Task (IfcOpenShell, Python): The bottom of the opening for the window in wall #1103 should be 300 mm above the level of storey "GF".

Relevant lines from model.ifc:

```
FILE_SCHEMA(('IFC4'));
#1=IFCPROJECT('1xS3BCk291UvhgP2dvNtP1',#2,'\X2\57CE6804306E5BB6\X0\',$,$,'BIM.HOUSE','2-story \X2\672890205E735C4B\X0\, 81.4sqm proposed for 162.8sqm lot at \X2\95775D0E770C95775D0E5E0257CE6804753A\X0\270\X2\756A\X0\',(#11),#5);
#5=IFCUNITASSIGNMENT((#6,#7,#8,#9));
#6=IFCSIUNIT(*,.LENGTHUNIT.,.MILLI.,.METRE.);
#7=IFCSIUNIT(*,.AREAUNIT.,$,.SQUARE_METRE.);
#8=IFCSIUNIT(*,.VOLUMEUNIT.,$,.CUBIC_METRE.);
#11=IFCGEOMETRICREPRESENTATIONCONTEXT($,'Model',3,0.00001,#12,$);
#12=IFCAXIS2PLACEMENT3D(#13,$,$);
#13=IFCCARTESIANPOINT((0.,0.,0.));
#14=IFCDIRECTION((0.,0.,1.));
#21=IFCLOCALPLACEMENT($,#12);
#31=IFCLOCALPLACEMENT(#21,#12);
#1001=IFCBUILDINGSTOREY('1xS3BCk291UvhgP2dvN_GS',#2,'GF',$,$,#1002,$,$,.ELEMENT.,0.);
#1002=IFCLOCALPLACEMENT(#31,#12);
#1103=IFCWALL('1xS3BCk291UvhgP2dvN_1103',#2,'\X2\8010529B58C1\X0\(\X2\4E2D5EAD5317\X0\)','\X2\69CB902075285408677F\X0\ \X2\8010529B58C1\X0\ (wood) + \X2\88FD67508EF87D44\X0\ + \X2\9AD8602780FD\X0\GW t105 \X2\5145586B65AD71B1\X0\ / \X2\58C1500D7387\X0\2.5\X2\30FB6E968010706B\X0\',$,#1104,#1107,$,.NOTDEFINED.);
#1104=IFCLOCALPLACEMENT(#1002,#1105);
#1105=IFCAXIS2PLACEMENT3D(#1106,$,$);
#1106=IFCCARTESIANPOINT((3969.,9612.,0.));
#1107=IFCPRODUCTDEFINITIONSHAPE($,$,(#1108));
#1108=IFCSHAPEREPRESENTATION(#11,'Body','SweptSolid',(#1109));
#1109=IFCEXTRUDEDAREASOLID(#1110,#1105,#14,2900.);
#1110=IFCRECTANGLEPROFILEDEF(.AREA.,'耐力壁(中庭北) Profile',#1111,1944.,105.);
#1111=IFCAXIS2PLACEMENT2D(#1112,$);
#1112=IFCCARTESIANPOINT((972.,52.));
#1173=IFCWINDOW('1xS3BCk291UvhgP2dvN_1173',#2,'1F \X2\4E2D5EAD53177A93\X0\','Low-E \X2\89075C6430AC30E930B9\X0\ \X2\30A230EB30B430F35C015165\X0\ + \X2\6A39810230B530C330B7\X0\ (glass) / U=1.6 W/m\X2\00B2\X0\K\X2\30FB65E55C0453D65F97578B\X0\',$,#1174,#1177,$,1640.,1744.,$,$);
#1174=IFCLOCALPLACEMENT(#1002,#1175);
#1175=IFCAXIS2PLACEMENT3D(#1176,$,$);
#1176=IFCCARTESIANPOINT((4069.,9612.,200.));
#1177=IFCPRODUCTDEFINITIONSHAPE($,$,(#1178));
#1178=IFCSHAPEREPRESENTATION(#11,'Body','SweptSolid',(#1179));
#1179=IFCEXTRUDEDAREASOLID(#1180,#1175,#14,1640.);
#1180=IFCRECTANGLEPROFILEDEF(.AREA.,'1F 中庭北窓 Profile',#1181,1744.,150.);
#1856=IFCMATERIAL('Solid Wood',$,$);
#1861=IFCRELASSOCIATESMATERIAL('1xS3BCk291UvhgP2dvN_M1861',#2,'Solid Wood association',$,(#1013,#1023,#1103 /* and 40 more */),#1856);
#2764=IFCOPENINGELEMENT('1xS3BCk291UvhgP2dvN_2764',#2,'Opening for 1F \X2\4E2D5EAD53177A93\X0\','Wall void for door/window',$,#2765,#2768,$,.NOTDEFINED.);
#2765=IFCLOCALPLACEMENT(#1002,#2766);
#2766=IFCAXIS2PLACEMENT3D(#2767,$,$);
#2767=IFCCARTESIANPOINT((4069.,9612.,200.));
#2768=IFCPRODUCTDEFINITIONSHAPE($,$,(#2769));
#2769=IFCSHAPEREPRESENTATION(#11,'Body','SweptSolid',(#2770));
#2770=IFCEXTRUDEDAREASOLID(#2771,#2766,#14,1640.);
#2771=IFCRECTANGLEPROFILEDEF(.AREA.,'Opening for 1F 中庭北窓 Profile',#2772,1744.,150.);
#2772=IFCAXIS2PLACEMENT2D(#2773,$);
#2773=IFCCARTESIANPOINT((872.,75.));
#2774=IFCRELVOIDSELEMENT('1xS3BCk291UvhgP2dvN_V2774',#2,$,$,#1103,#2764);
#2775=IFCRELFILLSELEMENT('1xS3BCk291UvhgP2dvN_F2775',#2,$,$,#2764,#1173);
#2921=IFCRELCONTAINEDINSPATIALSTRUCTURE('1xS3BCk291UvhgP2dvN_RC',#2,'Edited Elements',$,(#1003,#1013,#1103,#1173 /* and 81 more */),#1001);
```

```python
import numpy as np
import ifcopenshell
import ifcopenshell.api.geometry
import ifcopenshell.geom
import ifcopenshell.util.element
import ifcopenshell.util.placement
import ifcopenshell.util.shape
import ifcopenshell.util.unit

model = ifcopenshell.open("model.ifc")
unit_scale = ifcopenshell.util.unit.calculate_unit_scale(model)

window = model.by_guid("1xS3BCk291UvhgP2dvN_1173")
opening = window.FillsVoids[0].RelatingOpeningElement
storey = ifcopenshell.util.element.get_container(window, ifc_class="IfcBuildingStorey")
level = ifcopenshell.util.placement.get_local_placement(storey.ObjectPlacement)[2, 3]

# The opening's origin need not be at the sill, so measure its lowest point.
shape = ifcopenshell.geom.create_shape(ifcopenshell.geom.settings(), opening)
bottom = ifcopenshell.util.shape.get_shape_bottom_elevation(shape, shape.geometry) / unit_scale
dz = level + 0.3 / unit_scale - bottom

shift = np.array([0.0, 0.0, dz])
# The window is not placed relative to its opening, so move both.
for product in (opening, window):
    matrix = ifcopenshell.util.placement.get_local_placement(product.ObjectPlacement)
    matrix[:3, 3] += shift
    ifcopenshell.api.geometry.edit_object_placement(model, product=product, matrix=matrix, is_si=False)

print(f"moved by {dz * unit_scale:+.3f} m")

model.write("model_edited.ifc")
```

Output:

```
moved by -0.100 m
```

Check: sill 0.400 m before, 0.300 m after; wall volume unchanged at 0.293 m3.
